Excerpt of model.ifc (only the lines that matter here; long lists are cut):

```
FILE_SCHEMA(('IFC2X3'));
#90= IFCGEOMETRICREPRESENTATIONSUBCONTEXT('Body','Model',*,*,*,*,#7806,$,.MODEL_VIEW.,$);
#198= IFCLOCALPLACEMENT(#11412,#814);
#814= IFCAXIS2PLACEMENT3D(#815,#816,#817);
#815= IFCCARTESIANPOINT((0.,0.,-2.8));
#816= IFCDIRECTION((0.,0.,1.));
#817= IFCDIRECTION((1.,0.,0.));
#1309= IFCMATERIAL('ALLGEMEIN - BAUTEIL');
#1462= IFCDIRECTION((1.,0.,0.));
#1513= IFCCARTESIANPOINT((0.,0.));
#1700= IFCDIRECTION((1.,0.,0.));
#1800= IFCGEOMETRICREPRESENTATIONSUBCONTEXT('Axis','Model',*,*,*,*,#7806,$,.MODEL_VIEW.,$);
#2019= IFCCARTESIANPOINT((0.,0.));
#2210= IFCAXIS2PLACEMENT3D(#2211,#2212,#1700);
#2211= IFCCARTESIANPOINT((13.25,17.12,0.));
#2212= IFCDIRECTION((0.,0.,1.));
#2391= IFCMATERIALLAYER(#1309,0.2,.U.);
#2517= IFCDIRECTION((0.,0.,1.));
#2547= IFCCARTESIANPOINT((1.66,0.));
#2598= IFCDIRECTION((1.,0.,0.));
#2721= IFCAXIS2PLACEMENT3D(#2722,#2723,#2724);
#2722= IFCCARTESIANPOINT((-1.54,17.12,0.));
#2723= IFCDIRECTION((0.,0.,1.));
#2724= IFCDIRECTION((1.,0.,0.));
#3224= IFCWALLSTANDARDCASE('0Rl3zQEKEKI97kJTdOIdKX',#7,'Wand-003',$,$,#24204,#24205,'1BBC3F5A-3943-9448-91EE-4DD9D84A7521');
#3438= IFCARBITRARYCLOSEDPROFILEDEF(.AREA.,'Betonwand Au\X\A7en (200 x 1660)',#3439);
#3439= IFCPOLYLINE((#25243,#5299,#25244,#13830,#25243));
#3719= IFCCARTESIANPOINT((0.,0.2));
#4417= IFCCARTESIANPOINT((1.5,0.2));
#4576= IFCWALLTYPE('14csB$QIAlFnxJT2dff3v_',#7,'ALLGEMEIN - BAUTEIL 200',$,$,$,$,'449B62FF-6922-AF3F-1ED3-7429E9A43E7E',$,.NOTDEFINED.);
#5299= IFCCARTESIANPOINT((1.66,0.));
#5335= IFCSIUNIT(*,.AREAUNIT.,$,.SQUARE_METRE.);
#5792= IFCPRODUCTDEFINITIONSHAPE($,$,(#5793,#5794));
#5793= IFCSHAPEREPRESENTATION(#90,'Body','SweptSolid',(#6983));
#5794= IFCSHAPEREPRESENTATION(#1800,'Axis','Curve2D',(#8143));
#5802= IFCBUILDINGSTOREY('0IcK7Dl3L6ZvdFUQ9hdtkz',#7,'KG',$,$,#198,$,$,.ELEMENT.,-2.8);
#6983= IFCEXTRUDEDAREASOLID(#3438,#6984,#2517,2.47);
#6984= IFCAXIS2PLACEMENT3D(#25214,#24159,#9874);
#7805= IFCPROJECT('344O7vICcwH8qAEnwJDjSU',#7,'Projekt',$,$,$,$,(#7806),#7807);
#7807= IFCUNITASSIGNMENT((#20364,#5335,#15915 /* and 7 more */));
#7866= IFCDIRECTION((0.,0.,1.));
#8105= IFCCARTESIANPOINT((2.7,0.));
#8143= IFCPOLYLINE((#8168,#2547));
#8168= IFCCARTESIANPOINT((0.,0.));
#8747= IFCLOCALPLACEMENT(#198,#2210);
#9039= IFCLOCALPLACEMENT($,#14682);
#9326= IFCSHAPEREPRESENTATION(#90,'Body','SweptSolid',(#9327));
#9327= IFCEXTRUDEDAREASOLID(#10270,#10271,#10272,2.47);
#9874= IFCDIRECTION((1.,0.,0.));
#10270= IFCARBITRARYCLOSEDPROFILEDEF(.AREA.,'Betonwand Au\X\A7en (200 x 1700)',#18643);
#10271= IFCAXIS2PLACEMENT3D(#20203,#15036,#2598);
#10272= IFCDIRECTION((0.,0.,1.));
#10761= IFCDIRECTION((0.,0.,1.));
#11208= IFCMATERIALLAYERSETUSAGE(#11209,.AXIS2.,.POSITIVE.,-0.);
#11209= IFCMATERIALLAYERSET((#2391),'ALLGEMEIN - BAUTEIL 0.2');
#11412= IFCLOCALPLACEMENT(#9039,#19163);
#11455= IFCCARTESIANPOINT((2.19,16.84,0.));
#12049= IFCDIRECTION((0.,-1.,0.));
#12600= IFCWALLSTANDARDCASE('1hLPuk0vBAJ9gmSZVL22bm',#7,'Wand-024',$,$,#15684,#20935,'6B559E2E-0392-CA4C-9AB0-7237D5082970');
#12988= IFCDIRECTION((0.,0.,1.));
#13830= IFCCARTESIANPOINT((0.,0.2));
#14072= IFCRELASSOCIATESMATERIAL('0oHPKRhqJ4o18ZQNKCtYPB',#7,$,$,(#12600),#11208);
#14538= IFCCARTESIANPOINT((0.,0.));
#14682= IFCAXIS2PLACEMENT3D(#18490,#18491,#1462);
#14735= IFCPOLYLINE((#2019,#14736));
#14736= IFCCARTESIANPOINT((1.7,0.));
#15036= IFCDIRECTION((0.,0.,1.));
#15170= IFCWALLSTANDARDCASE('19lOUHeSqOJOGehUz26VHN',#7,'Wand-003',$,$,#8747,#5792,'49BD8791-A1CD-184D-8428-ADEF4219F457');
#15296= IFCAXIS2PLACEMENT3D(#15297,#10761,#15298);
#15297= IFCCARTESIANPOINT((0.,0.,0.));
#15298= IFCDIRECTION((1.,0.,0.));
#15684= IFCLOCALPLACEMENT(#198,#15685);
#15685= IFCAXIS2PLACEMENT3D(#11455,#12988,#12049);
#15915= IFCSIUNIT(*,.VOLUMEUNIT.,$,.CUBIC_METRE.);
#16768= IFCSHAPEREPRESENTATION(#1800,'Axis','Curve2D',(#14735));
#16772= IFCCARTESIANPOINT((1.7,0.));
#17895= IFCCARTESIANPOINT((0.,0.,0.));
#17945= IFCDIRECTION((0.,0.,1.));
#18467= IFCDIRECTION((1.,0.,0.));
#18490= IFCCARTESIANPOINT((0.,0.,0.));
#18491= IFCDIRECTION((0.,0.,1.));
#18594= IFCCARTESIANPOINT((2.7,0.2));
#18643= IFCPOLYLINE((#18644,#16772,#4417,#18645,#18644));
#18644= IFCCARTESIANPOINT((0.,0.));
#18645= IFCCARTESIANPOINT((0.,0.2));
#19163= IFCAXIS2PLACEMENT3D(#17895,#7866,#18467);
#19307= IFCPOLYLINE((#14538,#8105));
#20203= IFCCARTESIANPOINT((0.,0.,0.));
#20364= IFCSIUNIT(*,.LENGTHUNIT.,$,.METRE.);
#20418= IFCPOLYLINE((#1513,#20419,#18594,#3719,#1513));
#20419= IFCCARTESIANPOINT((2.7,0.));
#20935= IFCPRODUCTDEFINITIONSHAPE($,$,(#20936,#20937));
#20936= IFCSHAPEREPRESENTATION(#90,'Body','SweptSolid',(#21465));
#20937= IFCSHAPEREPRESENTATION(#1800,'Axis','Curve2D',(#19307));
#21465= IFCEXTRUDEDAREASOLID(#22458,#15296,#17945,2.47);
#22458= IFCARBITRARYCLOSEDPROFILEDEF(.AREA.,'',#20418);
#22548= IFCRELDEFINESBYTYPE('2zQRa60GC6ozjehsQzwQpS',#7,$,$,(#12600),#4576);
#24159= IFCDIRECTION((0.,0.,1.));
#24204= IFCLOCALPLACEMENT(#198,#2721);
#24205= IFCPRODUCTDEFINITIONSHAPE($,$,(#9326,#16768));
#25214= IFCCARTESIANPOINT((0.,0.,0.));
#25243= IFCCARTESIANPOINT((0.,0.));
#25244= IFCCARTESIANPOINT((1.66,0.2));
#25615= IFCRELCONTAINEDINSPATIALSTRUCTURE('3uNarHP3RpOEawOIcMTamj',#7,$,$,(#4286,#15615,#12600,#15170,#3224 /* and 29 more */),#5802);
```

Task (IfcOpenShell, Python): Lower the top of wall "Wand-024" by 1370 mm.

```python
import ifcopenshell
import ifcopenshell.geom
import ifcopenshell.util.representation
import ifcopenshell.util.shape
import ifcopenshell.util.unit

model = ifcopenshell.open("model.ifc")
unit_scale = ifcopenshell.util.unit.calculate_unit_scale(model)
settings = ifcopenshell.geom.settings()


def volume(element):
    """Net volume in cubic metres, openings subtracted."""
    shape = ifcopenshell.geom.create_shape(settings, element)
    return ifcopenshell.util.shape.get_volume(shape.geometry)


wall = model.by_guid("1hLPuk0vBAJ9gmSZVL22bm")
before = volume(wall)

body = ifcopenshell.util.representation.get_representation(wall, "Model", "Body")
solid = body.Items[0]
old_height = solid.Depth
solid.Depth -= 1.37 / unit_scale
after = volume(wall)

print(f"height {old_height:g} -> {solid.Depth:g}, volume {before:.3f} -> {after:.3f} m3")

model.write("model_v2.ifc")
```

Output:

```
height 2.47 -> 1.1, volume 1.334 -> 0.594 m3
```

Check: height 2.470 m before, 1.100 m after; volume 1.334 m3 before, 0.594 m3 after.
